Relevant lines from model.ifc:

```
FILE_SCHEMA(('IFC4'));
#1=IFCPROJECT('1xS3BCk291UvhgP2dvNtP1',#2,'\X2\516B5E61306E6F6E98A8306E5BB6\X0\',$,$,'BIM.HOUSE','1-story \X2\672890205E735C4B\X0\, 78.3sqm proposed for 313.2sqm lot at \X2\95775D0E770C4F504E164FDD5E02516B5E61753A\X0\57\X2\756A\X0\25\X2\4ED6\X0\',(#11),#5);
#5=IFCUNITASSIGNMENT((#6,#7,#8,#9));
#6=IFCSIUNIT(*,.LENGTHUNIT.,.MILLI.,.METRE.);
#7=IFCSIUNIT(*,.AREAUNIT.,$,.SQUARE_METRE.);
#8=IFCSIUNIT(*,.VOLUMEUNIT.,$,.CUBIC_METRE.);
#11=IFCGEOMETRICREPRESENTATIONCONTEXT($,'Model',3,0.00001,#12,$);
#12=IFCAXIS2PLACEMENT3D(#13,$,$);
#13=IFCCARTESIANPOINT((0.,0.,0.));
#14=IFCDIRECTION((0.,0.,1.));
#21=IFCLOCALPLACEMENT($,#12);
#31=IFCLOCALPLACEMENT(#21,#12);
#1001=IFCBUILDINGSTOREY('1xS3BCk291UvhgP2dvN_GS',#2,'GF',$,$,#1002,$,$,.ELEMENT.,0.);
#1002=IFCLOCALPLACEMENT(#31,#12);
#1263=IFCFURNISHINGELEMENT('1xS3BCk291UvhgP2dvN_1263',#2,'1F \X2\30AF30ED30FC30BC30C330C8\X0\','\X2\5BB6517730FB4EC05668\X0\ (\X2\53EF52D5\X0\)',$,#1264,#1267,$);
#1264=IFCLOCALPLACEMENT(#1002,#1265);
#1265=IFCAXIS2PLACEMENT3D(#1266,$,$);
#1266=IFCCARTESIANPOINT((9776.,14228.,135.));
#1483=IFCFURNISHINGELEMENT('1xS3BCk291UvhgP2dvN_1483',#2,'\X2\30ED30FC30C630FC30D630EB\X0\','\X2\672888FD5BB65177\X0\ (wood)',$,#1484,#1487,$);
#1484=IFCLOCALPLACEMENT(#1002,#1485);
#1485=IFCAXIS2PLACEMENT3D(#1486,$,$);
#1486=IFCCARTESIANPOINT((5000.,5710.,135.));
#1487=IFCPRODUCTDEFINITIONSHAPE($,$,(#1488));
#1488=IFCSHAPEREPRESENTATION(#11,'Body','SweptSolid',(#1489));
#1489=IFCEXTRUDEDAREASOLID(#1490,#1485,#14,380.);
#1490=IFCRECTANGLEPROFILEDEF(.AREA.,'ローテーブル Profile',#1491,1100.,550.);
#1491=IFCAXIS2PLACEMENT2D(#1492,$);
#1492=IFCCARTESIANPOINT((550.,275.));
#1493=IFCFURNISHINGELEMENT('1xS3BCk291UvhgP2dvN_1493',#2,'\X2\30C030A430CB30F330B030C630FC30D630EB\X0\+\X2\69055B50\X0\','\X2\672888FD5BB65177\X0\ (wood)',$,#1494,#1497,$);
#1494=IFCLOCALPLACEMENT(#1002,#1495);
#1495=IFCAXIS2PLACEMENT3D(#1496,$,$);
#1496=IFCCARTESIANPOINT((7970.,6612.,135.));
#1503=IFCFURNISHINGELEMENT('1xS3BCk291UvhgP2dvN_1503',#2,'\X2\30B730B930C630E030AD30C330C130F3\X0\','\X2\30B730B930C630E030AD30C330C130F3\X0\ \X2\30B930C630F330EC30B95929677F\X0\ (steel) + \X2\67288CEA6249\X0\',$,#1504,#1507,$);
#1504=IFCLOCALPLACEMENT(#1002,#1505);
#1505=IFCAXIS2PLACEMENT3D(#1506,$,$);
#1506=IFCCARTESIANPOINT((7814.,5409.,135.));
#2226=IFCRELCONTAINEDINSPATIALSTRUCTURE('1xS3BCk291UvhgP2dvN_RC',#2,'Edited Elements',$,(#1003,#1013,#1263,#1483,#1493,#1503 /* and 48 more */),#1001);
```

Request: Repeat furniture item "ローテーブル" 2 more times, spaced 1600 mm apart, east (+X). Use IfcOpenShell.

```python
import numpy as np
import ifcopenshell
import ifcopenshell.api.geometry
import ifcopenshell.api.root
import ifcopenshell.util.element
import ifcopenshell.util.placement
import ifcopenshell.util.unit

model = ifcopenshell.open("model.ifc")
unit_scale = ifcopenshell.util.unit.calculate_unit_scale(model)


def reuse_history(source, copy):
    """copy_class also copies each property set's owner history, people and application; keep the originals."""
    for rel in copy.IsDefinedBy:
        if rel.is_a("IfcRelDefinesByProperties") and (history := rel.RelatingPropertyDefinition.OwnerHistory):
            rel.RelatingPropertyDefinition.OwnerHistory = source.OwnerHistory
            ifcopenshell.util.element.remove_deep2(model, history)


source = model.by_guid("1xS3BCk291UvhgP2dvN_1483")
base = ifcopenshell.util.placement.get_local_placement(source.ObjectPlacement)
step = np.array([1.0, 0.0, 0.0]) * 1.6 / unit_scale

for i in range(1, 3):
    copy = ifcopenshell.api.root.copy_class(model, product=source)
    copy.Representation = ifcopenshell.util.element.copy_deep(
        model, source.Representation, exclude=["IfcGeometricRepresentationContext", "IfcRepresentationMap"]
    )
    reuse_history(source, copy)
    matrix = base.copy()
    matrix[:3, 3] += i * step
    print("added at", matrix[:3, 3].round(3) + 0.0)
    ifcopenshell.api.geometry.edit_object_placement(model, product=copy, matrix=matrix, is_si=False)

model.write("model_edited.ifc")
```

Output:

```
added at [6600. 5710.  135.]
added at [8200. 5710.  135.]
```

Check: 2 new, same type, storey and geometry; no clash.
